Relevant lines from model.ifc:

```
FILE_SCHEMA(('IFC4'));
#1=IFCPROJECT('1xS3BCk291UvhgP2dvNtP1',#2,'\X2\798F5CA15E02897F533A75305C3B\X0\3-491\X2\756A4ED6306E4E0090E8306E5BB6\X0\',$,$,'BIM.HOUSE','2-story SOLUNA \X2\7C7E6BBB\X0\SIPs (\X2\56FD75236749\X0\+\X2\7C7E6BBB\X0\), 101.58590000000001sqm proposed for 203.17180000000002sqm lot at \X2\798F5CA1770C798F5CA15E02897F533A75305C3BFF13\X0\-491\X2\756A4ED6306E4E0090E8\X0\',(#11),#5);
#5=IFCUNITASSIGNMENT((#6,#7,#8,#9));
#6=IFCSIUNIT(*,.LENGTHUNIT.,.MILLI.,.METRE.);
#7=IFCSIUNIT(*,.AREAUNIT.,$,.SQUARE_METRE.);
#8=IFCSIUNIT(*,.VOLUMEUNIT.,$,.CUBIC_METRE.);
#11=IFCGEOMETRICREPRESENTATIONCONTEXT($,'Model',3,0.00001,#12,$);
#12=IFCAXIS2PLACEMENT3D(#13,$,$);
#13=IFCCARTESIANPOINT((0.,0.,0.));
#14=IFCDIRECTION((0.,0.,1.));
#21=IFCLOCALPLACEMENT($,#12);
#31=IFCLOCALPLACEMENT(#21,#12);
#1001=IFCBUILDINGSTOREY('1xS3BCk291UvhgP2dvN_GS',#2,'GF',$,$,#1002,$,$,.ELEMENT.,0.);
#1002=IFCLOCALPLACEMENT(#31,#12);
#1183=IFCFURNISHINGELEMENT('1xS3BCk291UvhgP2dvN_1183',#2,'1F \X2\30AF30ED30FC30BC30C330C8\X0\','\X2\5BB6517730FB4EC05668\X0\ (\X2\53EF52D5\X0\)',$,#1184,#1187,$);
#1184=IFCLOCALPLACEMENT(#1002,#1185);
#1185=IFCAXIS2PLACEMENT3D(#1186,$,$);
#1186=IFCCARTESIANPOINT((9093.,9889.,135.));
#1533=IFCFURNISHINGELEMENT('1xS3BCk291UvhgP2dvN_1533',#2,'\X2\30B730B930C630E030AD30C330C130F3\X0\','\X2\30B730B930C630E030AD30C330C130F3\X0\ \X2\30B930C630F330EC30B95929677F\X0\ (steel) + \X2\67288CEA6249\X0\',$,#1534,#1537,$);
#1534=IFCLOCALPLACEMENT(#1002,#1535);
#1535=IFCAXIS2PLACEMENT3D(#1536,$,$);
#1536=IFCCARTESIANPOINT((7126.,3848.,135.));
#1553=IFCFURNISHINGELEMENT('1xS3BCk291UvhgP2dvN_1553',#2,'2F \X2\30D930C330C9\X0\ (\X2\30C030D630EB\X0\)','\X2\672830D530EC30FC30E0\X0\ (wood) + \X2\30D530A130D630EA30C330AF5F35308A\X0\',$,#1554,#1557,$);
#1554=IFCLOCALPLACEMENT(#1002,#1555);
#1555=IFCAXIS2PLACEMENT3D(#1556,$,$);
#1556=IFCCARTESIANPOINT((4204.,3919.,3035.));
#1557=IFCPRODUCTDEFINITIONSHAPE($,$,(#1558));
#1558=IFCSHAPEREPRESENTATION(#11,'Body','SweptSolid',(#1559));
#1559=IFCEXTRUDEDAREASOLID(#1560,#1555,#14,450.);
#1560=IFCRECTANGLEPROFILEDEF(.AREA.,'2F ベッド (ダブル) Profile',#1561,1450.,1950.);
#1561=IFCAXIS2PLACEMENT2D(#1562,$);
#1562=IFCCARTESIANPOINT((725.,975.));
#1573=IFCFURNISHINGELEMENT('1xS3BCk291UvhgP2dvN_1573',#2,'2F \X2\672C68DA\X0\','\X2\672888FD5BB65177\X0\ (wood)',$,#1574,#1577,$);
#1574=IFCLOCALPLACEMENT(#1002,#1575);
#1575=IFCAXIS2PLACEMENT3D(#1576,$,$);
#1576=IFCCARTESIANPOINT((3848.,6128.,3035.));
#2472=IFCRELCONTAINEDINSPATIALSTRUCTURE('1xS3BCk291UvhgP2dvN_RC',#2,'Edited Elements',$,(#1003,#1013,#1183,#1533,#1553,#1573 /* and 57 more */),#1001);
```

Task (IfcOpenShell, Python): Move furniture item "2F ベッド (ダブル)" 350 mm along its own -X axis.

```python
import ifcopenshell
import ifcopenshell.api.geometry
import ifcopenshell.util.placement
import ifcopenshell.util.unit

model = ifcopenshell.open("model.ifc")
unit_scale = ifcopenshell.util.unit.calculate_unit_scale(model)

item = model.by_id(1553)
matrix = ifcopenshell.util.placement.get_local_placement(item.ObjectPlacement)
matrix[:3, 3] -= matrix[:3, 0] * 0.35 / unit_scale
ifcopenshell.api.geometry.edit_object_placement(model, product=item, matrix=matrix, is_si=False)

print(ifcopenshell.util.placement.get_local_placement(item.ObjectPlacement).round(3) + 0.0)

model.write("model_updated.ifc")
```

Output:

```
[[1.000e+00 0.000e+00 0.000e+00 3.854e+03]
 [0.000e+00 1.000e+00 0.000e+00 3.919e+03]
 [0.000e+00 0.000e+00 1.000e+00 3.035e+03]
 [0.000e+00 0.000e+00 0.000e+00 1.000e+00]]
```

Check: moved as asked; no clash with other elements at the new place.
